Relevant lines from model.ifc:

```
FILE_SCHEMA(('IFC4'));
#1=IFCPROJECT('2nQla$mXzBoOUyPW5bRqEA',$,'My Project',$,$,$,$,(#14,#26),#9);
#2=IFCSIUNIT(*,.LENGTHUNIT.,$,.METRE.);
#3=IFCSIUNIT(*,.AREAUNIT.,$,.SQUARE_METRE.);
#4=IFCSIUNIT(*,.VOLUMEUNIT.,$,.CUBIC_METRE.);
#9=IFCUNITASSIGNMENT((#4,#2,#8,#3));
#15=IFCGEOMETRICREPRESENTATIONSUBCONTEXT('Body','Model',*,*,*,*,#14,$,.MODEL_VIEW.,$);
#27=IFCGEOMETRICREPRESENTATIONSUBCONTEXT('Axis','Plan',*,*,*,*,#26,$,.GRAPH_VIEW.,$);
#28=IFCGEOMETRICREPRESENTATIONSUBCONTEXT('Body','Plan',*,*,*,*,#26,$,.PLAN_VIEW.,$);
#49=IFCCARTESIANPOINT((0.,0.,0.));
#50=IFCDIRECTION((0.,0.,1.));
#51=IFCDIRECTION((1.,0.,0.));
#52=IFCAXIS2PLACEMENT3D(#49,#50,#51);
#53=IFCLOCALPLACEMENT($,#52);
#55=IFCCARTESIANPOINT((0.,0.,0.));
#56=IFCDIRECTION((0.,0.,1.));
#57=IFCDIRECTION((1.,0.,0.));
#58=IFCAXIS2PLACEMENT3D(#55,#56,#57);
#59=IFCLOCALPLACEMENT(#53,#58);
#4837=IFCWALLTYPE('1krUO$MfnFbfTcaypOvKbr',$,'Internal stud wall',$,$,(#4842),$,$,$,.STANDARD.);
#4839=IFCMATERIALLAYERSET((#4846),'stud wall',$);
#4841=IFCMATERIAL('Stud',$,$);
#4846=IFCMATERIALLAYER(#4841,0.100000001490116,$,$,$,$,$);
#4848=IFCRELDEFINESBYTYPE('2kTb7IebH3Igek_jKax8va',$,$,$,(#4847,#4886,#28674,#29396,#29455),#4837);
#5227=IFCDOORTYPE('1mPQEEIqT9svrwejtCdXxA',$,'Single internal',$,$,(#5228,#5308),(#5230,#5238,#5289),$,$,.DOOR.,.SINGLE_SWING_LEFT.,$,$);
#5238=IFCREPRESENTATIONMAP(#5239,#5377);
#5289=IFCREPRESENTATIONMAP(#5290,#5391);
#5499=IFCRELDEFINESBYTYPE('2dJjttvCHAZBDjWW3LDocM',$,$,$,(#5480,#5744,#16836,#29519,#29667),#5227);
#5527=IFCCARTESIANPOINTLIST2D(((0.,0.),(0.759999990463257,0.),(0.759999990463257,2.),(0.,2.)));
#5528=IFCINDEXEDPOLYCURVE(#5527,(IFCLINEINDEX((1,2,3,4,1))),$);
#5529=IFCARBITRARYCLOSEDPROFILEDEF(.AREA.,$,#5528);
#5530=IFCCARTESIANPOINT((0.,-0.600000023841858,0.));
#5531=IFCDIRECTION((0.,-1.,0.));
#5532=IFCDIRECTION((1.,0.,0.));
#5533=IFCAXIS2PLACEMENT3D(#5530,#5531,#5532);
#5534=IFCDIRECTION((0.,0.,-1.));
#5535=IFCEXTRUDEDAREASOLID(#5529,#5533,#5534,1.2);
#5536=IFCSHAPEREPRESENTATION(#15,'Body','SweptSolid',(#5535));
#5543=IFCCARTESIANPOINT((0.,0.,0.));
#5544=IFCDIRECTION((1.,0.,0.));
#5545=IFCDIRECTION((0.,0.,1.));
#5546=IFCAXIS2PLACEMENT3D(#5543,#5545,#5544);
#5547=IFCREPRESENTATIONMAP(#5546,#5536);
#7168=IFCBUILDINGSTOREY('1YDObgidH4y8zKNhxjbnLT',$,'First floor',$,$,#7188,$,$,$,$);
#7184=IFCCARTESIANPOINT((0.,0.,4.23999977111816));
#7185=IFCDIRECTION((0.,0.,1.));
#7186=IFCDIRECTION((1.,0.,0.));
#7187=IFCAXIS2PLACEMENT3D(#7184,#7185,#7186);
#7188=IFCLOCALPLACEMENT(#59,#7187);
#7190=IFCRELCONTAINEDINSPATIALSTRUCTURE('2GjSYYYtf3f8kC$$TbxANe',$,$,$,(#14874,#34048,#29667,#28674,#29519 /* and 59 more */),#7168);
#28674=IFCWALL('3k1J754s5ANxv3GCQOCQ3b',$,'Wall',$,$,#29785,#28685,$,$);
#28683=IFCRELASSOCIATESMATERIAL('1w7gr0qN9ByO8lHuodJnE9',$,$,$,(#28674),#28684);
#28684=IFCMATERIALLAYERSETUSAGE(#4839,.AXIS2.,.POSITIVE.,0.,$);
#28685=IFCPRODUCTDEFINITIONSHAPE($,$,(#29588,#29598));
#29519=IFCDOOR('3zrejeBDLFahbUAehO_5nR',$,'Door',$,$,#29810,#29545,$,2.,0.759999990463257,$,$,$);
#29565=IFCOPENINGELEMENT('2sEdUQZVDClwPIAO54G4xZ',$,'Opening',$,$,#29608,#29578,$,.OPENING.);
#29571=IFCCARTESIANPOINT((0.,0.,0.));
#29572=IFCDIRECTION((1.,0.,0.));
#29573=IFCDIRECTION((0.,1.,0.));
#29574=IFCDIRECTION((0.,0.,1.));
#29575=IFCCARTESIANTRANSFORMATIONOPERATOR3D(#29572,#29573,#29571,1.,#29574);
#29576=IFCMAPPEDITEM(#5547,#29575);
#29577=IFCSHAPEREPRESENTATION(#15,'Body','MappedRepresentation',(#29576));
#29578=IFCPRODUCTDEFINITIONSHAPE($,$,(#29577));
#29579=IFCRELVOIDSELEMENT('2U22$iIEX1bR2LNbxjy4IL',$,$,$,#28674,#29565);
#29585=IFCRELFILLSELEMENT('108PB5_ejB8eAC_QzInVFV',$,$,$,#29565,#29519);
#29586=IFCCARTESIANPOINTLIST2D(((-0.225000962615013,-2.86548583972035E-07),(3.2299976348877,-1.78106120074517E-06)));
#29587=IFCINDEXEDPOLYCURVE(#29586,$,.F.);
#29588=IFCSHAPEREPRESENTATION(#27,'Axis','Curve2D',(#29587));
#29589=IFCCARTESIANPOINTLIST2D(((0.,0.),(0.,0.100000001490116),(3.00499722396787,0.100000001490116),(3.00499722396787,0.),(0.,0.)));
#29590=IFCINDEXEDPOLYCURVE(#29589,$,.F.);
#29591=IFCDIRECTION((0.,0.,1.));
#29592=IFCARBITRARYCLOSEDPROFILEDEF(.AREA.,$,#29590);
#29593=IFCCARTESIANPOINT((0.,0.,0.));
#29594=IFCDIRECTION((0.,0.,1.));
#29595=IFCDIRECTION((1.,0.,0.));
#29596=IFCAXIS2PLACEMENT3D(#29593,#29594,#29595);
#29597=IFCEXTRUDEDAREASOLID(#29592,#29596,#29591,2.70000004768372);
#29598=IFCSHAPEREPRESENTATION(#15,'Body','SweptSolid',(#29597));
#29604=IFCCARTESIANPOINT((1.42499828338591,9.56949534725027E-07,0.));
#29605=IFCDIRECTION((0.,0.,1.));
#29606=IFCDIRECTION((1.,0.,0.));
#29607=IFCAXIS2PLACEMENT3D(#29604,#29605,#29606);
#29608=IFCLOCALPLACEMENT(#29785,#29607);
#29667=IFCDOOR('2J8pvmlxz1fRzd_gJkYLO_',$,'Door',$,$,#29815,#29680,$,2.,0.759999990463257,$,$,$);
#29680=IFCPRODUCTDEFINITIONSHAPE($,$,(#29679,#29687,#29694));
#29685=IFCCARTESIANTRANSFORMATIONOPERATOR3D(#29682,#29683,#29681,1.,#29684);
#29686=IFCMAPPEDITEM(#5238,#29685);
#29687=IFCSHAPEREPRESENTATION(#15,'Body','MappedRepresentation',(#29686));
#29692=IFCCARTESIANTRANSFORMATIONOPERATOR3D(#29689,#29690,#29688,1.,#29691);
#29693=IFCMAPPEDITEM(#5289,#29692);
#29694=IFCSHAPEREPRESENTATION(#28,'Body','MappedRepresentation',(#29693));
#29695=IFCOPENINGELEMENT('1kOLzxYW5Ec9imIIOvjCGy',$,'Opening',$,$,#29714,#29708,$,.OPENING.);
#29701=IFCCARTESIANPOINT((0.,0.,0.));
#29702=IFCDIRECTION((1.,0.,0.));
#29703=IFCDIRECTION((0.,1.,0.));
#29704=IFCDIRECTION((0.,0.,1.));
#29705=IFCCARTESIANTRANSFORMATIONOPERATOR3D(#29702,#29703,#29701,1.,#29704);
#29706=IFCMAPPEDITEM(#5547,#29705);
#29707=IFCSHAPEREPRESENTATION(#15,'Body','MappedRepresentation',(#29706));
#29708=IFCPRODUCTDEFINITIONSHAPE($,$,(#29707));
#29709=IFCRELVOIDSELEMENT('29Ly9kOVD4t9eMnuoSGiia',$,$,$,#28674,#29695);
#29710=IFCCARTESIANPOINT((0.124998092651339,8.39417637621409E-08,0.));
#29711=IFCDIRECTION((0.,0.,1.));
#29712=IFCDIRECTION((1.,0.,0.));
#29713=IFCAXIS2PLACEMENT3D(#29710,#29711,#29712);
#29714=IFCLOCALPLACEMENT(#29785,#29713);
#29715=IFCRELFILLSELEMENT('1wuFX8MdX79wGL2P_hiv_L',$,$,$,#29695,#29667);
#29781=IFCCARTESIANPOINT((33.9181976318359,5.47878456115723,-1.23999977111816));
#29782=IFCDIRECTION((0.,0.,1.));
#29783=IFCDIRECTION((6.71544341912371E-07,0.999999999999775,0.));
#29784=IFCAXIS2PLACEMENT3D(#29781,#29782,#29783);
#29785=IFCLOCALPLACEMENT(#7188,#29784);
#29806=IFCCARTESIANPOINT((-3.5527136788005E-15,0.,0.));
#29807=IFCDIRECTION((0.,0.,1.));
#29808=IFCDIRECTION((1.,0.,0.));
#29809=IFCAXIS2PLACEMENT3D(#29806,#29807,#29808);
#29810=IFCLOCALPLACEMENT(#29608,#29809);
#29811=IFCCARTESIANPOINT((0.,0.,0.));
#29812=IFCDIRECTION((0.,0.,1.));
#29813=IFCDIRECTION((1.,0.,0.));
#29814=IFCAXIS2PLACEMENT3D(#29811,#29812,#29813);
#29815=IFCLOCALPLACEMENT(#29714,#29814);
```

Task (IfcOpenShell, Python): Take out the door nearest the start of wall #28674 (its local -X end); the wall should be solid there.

```python
import ifcopenshell
import ifcopenshell.api.feature
import ifcopenshell.api.root
import ifcopenshell.geom
import ifcopenshell.util.shape

model = ifcopenshell.open("model.ifc")
settings = ifcopenshell.geom.settings()


def volume(element):
    """Net volume in cubic metres, openings subtracted."""
    shape = ifcopenshell.geom.create_shape(settings, element)
    return ifcopenshell.util.shape.get_volume(shape.geometry)


door = model.by_id(29667)
opening = door.FillsVoids[0].RelatingOpeningElement
wall = opening.VoidsElements[0].RelatingBuildingElement
before = volume(wall)

ifcopenshell.api.root.remove_product(model, product=door)
ifcopenshell.api.feature.remove_feature(model, feature=opening)

after = volume(wall)

print(f"wall volume {before:.3f} -> {after:.3f} m3")

model.write("model_v2.ifc")
```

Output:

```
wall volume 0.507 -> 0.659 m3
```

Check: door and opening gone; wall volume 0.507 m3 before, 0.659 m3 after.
